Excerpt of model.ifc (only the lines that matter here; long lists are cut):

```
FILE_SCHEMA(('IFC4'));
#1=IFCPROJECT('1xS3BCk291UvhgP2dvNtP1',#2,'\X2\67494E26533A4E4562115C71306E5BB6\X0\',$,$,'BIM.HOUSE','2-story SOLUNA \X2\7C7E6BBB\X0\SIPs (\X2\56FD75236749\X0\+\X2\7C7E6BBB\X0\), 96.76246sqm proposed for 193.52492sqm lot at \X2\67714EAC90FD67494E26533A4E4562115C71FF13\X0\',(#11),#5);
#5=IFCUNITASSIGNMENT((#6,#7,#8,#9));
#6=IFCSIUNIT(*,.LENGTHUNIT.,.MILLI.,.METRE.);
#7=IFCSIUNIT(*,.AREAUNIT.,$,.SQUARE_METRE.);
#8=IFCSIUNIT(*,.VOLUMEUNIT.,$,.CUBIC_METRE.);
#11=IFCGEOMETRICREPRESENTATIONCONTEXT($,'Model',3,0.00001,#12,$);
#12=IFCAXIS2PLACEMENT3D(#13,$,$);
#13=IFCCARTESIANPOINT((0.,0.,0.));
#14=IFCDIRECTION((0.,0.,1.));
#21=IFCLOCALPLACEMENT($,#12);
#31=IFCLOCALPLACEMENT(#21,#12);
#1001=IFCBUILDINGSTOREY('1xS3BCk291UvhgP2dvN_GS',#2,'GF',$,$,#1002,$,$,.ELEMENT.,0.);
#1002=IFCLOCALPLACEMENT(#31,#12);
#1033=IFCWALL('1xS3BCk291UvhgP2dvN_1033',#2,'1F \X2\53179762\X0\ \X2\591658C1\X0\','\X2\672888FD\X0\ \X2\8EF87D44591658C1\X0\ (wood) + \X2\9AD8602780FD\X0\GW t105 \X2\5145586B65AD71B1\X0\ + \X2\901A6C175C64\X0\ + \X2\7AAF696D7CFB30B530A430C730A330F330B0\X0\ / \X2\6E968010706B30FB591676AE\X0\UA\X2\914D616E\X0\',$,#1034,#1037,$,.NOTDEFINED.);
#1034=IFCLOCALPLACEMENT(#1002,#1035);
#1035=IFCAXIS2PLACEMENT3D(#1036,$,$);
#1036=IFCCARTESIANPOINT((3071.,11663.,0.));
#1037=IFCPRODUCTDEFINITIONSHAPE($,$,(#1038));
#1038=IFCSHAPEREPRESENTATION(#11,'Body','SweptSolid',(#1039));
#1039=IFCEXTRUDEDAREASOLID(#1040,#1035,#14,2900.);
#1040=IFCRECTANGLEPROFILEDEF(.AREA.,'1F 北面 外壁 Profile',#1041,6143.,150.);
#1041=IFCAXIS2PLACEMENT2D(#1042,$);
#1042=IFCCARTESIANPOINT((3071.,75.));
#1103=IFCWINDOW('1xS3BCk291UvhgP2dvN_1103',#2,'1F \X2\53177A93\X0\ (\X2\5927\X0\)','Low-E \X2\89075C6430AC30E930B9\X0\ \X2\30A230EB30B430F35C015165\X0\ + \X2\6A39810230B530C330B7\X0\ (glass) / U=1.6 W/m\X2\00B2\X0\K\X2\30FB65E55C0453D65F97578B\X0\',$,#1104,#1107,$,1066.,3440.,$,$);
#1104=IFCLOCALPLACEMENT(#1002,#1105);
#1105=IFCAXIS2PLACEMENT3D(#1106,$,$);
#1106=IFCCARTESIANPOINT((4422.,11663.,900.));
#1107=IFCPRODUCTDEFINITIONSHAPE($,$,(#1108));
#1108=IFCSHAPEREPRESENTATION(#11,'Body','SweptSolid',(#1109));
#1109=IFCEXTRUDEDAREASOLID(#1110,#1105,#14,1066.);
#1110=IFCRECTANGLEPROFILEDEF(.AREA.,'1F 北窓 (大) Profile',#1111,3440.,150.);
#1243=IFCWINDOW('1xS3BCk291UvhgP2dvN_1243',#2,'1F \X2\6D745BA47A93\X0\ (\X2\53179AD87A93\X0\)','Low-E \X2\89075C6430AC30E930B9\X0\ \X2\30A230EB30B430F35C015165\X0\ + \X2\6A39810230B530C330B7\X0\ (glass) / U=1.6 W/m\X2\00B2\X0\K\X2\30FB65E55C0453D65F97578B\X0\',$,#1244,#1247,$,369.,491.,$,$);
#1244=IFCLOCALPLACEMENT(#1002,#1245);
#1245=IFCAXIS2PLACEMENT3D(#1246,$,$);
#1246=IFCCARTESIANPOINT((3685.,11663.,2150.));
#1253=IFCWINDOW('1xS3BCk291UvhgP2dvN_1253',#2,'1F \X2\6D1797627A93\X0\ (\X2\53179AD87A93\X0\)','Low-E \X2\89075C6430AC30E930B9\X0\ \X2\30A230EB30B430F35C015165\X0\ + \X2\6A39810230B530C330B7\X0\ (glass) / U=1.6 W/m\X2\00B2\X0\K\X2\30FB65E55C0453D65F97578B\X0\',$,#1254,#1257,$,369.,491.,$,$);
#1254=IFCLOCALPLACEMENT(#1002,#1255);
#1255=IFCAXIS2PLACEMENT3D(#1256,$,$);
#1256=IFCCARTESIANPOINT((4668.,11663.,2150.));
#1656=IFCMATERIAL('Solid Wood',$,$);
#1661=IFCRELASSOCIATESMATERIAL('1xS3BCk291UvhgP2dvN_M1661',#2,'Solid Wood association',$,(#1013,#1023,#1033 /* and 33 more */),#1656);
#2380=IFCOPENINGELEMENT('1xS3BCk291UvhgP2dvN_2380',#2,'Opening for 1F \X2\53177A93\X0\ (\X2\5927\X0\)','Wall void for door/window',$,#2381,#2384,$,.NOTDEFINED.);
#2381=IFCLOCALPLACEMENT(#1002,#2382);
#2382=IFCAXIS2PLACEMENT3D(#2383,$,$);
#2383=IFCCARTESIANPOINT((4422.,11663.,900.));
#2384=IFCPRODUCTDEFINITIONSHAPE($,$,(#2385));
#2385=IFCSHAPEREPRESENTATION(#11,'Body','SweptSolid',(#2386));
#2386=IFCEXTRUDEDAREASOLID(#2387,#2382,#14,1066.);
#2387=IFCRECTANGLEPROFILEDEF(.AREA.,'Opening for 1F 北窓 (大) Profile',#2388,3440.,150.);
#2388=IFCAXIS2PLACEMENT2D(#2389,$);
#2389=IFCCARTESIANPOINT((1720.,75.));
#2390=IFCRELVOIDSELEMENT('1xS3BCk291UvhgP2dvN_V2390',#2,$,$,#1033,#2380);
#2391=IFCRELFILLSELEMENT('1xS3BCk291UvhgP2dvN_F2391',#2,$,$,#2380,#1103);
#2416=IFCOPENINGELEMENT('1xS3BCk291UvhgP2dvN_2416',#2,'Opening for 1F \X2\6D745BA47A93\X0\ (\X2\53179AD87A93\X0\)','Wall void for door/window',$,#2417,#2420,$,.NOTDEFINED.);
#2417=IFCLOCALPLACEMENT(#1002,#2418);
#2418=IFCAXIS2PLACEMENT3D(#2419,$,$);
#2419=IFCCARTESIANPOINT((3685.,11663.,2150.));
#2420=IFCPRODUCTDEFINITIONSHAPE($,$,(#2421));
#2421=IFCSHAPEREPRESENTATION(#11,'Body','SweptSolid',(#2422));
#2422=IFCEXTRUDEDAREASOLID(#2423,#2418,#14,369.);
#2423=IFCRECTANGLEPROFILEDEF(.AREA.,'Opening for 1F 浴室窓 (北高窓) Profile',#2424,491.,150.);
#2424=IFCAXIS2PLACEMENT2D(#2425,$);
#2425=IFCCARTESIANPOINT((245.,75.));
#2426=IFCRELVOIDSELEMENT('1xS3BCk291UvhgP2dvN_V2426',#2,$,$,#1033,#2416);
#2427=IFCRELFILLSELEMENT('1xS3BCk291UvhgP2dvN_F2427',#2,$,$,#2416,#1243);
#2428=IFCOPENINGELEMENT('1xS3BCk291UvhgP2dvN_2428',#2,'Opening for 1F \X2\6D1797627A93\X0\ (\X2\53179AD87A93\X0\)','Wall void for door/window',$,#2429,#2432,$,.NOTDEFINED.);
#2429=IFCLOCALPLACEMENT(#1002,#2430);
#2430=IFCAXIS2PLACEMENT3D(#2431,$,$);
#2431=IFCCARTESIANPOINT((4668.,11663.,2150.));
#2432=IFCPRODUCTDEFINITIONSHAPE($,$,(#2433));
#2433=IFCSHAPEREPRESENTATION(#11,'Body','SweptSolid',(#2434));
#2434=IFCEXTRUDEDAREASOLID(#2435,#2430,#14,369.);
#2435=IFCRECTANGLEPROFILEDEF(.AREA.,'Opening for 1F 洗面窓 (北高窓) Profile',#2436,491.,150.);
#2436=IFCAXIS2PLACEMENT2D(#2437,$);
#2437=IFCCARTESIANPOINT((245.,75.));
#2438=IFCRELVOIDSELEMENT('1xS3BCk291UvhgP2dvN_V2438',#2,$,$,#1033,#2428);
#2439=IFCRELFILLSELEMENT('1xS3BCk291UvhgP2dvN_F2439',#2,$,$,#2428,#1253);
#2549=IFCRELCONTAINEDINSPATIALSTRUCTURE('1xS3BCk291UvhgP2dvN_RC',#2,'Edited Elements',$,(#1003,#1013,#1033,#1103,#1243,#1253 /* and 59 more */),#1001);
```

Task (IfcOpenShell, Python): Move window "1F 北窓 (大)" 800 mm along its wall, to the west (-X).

```python
import ifcopenshell
import ifcopenshell.api.geometry
import ifcopenshell.util.placement
import ifcopenshell.util.unit

model = ifcopenshell.open("model.ifc")
unit_scale = ifcopenshell.util.unit.calculate_unit_scale(model)

window = model.by_guid("1xS3BCk291UvhgP2dvN_1103")
opening = window.FillsVoids[0].RelatingOpeningElement
wall = opening.VoidsElements[0].RelatingBuildingElement

wall_matrix = ifcopenshell.util.placement.get_local_placement(wall.ObjectPlacement)
shift = wall_matrix[:3, 0] * -0.8 / unit_scale
before = ifcopenshell.util.placement.get_local_placement(window.ObjectPlacement)[:3, 3].copy()

# The window is not placed relative to its opening, so move both.
for product in (opening, window):
    matrix = ifcopenshell.util.placement.get_local_placement(product.ObjectPlacement)
    matrix[:3, 3] += shift
    ifcopenshell.api.geometry.edit_object_placement(model, product=product, matrix=matrix, is_si=False)

after = ifcopenshell.util.placement.get_local_placement(window.ObjectPlacement)[:3, 3]
print("window moved by", (after - before).round(3) + 0.0)

model.write("model_v2.ifc")
```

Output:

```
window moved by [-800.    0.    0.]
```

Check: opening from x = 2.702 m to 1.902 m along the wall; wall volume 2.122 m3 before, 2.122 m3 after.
